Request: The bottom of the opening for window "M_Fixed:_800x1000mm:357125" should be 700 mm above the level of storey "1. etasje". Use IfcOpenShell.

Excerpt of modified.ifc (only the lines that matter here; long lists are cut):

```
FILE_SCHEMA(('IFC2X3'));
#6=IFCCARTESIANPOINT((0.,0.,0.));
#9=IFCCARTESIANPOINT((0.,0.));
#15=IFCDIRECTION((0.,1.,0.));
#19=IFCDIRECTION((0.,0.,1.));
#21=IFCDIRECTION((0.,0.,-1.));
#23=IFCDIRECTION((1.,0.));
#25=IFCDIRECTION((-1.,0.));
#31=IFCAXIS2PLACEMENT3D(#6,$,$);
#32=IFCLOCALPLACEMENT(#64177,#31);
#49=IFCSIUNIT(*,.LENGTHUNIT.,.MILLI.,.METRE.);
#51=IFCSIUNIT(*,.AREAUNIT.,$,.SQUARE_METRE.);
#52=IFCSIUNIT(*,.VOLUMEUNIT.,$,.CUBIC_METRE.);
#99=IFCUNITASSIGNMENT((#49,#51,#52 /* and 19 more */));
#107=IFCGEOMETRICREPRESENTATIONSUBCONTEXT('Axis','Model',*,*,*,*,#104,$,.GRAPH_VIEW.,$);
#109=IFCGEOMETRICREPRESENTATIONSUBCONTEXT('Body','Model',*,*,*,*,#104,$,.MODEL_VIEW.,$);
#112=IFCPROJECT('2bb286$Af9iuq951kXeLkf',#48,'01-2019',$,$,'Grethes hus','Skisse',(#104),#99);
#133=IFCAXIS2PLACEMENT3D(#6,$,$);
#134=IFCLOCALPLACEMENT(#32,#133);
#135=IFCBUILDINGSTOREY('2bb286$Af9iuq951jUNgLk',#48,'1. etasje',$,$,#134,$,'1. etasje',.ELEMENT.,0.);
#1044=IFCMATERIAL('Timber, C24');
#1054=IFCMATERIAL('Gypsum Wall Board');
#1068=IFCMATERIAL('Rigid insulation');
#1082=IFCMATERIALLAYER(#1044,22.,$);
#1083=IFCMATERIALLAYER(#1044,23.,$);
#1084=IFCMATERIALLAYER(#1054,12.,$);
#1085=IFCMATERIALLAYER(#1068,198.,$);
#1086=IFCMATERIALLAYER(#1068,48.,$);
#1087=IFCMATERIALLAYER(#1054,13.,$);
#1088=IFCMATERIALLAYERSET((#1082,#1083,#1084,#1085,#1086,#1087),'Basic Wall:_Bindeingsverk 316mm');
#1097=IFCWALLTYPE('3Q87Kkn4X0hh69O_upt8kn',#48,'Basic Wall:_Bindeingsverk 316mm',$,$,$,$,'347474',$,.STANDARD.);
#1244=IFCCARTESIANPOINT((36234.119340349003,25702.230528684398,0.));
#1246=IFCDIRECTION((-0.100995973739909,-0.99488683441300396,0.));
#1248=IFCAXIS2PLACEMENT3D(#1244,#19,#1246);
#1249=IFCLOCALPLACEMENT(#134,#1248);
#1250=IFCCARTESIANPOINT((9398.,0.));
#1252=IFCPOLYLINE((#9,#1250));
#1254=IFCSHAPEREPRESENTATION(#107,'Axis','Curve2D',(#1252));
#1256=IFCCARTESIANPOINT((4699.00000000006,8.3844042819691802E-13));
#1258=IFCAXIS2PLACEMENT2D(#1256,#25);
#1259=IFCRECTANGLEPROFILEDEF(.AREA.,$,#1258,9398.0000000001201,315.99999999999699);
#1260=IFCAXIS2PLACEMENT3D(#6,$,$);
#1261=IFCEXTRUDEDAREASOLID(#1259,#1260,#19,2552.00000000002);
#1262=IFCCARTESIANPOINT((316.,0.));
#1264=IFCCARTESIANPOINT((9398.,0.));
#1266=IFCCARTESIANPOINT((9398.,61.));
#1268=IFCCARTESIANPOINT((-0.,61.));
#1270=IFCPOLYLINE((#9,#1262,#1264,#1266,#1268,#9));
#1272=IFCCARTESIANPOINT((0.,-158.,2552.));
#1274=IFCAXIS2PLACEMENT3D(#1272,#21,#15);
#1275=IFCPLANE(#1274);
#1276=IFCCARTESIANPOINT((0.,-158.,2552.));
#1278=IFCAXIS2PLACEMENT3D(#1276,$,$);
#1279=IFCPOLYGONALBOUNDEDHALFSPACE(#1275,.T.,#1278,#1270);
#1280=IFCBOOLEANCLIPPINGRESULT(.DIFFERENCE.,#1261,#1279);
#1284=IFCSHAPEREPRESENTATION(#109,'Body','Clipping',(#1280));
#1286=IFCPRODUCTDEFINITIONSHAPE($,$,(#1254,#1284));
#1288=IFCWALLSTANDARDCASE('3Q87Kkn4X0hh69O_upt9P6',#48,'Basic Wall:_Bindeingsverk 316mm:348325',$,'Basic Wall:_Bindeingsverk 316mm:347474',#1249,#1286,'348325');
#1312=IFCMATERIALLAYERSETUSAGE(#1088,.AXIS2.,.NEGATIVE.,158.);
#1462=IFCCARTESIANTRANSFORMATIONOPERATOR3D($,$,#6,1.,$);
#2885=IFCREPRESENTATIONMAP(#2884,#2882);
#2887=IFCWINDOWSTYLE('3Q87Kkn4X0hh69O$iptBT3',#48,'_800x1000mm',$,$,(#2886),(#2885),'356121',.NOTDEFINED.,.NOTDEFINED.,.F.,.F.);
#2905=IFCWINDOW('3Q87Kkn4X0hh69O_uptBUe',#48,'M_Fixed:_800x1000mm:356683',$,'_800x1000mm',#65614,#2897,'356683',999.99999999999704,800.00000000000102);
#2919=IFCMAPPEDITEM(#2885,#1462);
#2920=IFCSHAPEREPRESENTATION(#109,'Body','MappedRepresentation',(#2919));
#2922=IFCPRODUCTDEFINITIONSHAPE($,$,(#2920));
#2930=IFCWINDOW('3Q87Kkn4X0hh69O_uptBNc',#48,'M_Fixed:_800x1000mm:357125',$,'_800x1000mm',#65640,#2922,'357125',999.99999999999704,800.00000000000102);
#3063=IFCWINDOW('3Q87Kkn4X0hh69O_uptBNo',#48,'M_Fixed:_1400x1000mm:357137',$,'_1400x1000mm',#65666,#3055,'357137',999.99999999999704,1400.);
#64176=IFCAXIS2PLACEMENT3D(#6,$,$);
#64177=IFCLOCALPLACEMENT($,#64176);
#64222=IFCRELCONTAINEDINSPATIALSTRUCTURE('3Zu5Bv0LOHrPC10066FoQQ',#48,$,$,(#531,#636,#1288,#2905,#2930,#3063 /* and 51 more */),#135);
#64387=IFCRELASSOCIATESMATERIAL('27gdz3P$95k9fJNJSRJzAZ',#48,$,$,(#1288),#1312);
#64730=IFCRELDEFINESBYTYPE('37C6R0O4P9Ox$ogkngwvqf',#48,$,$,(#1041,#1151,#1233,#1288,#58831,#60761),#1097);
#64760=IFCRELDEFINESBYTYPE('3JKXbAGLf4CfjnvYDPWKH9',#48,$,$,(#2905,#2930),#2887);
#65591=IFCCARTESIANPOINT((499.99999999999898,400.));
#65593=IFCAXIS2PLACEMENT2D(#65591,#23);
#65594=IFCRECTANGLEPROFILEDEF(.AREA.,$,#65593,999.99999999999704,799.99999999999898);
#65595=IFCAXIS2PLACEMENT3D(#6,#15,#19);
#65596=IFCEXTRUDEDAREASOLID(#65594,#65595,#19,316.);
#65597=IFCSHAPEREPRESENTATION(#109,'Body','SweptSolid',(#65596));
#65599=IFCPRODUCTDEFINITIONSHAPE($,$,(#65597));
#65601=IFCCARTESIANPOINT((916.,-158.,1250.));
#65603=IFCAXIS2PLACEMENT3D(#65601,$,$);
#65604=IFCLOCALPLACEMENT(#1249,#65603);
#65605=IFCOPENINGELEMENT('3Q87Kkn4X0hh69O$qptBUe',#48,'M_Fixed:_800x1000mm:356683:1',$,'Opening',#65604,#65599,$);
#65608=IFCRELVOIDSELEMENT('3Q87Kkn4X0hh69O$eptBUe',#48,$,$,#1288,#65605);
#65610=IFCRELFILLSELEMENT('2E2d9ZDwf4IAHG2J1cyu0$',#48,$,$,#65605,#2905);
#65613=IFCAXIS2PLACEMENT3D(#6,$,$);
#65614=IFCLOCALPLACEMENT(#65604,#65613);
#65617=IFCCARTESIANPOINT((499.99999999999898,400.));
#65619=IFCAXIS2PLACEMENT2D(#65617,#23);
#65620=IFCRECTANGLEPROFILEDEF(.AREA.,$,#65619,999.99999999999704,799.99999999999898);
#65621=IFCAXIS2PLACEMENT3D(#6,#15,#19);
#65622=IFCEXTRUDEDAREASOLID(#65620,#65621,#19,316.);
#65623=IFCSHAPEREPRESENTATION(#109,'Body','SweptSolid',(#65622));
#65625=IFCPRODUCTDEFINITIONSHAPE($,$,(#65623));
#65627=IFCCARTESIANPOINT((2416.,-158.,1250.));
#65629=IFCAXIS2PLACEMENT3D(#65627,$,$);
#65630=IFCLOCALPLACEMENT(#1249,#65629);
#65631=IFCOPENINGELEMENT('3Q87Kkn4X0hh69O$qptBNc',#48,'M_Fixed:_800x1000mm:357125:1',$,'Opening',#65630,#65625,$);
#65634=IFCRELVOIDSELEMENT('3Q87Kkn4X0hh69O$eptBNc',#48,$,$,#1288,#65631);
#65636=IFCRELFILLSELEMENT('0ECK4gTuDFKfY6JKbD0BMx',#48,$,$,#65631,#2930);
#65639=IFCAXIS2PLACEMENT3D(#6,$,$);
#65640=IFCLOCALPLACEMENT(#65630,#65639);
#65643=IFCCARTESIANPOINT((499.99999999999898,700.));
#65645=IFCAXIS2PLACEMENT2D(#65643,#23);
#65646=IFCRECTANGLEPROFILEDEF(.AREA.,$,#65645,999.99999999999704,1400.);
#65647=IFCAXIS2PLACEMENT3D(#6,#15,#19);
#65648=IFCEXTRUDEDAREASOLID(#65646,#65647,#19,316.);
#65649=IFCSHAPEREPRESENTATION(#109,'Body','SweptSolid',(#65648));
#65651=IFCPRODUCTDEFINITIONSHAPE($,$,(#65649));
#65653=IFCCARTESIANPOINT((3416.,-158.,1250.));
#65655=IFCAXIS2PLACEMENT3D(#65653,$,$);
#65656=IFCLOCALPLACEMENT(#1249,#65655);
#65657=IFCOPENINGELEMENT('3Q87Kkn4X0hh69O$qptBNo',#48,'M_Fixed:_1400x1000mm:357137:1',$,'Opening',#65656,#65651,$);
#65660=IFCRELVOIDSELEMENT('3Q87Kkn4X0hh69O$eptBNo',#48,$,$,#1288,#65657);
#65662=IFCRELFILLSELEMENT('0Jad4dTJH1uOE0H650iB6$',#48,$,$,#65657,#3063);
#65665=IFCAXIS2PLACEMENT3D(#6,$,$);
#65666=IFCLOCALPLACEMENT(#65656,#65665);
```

```python
import numpy as np
import ifcopenshell
import ifcopenshell.api.geometry
import ifcopenshell.geom
import ifcopenshell.util.element
import ifcopenshell.util.placement
import ifcopenshell.util.shape
import ifcopenshell.util.unit

model = ifcopenshell.open("modified.ifc")
unit_scale = ifcopenshell.util.unit.calculate_unit_scale(model)

window = model.by_guid("3Q87Kkn4X0hh69O_uptBNc")
opening = window.FillsVoids[0].RelatingOpeningElement
storey = ifcopenshell.util.element.get_container(window, ifc_class="IfcBuildingStorey")
level = ifcopenshell.util.placement.get_local_placement(storey.ObjectPlacement)[2, 3]

# The opening's origin need not be at the sill, so measure its lowest point.
shape = ifcopenshell.geom.create_shape(ifcopenshell.geom.settings(), opening)
bottom = ifcopenshell.util.shape.get_shape_bottom_elevation(shape, shape.geometry) / unit_scale
dz = level + 700.0 - bottom

shift = np.array([0.0, 0.0, dz])
# The window is placed relative to its opening, so it follows when the opening moves.
matrix = ifcopenshell.util.placement.get_local_placement(opening.ObjectPlacement)
matrix[:3, 3] += shift
ifcopenshell.api.geometry.edit_object_placement(
    model, product=opening, matrix=matrix, is_si=False, should_transform_children=True
)

print(f"moved by {dz * unit_scale:+.3f} m")

model.write("modified-out.ifc")
```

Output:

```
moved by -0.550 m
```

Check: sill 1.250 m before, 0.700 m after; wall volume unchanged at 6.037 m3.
